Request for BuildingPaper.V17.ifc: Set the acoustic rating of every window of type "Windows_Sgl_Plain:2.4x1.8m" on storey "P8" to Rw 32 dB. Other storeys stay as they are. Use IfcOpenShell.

First a look at what the model holds.

```python
import ifcopenshell
import ifcopenshell.util.element

model = ifcopenshell.open("BuildingPaper.V17.ifc")
print(model.schema)
storey = next(s for s in model.by_type("IfcBuildingStorey") if s.Name == "P8")
windows = [e for e in ifcopenshell.util.element.get_decomposition(storey) if e.is_a("IfcWindow")]
seen = {}
for e in windows:
    element_type = ifcopenshell.util.element.get_type(e)
    key = (element_type.Name if element_type != e and element_type else None, ifcopenshell.util.element.get_pset(e, "Pset_WindowCommon", "AcousticRating"))
    seen[key] = seen.get(key, 0) + 1
for (name, value), count in sorted(seen.items(), key=str):
    print(count, "x", name, "|", value)
```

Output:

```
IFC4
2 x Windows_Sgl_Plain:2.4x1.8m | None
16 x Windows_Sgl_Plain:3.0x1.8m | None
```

```python
import ifcopenshell
import ifcopenshell.api.pset
import ifcopenshell.util.element

model = ifcopenshell.open("BuildingPaper.V17.ifc")

storey = next(s for s in model.by_type("IfcBuildingStorey") if s.Name == "P8")
windows = [e for e in ifcopenshell.util.element.get_decomposition(storey) if e.is_a("IfcWindow")]

count = 0
for e in windows:
    element_type = ifcopenshell.util.element.get_type(e)
    if element_type in (None, e) or element_type.Name != "Windows_Sgl_Plain:2.4x1.8m":
        continue
    # add_pset returns the element's existing set when there is one.
    pset = ifcopenshell.api.pset.add_pset(model, product=e, name="Pset_WindowCommon")
    ifcopenshell.api.pset.edit_pset(model, pset=pset, properties={"AcousticRating": "Rw 32 dB"})
    count += 1

print(count, "windows updated")

model.write("BuildingPaper.V17_rev.ifc")
```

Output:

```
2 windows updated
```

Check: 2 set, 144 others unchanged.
